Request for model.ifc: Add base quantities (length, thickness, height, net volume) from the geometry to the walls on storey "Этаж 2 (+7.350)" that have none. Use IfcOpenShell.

First a look at what the model holds.

```python
import ifcopenshell
import ifcopenshell.util.element
import ifcopenshell.util.unit

model = ifcopenshell.open("model.ifc")
print(model.schema)
for unit_type in ("LENGTHUNIT", "AREAUNIT", "VOLUMEUNIT"):
    print(unit_type, ifcopenshell.util.unit.calculate_unit_scale(model, unit_type))
storey = next(s for s in model.by_type("IfcBuildingStorey") if s.Name == "Этаж 2 (+7.350)")
walls = [e for e in ifcopenshell.util.element.get_decomposition(storey) if e.is_a("IfcWall")]
for e in sorted(walls, key=lambda e: e.id()):
    print(e.id(), e.is_a(), e.Name, list(ifcopenshell.util.element.get_psets(e, qtos_only=True)), sep=" | ")
```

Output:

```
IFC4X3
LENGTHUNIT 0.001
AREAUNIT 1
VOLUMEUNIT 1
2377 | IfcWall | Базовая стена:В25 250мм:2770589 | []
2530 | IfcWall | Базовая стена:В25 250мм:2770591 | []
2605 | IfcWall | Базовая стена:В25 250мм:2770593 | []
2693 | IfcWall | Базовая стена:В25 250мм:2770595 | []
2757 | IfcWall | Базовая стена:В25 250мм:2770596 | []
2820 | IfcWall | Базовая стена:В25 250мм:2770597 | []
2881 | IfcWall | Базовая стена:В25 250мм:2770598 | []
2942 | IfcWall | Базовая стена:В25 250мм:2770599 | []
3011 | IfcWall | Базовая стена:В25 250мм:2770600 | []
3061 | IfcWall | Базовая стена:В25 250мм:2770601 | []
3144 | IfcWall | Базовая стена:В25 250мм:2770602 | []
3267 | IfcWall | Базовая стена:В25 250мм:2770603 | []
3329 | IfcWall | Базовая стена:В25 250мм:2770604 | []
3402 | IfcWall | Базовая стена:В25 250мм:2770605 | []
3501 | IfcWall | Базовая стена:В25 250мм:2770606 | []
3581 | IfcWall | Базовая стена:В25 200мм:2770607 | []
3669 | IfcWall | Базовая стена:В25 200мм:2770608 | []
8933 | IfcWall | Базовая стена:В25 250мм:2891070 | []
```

```python
import ifcopenshell
import ifcopenshell.api.pset
import ifcopenshell.geom
import ifcopenshell.util.element
import ifcopenshell.util.shape
import ifcopenshell.util.unit

model = ifcopenshell.open("model.ifc")
unit_scale = ifcopenshell.util.unit.calculate_unit_scale(model)
volume_scale = ifcopenshell.util.unit.calculate_unit_scale(model, "VOLUMEUNIT")
settings = ifcopenshell.geom.settings()

storey = next(s for s in model.by_type("IfcBuildingStorey") if s.Name == "Этаж 2 (+7.350)")
walls = [e for e in ifcopenshell.util.element.get_decomposition(storey) if e.is_a("IfcWall")]

for e in sorted(walls, key=lambda e: e.id()):
    if ifcopenshell.util.element.get_psets(e, qtos_only=True, should_inherit=False):
        continue
    # Geometry comes back in metres, in the element's own axes.
    shape = ifcopenshell.geom.create_shape(settings, e)
    values = {
        "Length": ifcopenshell.util.shape.get_x(shape.geometry) / unit_scale,
        "Width": ifcopenshell.util.shape.get_y(shape.geometry) / unit_scale,
        "Height": ifcopenshell.util.shape.get_z(shape.geometry) / unit_scale,
        "NetVolume": ifcopenshell.util.shape.get_volume(shape.geometry) / volume_scale,
    }
    qto = ifcopenshell.api.pset.add_qto(model, product=e, name="Qto_WallBaseQuantities")
    ifcopenshell.api.pset.edit_qto(model, qto=qto, properties=values)
    print(e.id(), {k: round(v, 3) for k, v in values.items()})

model.write("model-out.ifc")
```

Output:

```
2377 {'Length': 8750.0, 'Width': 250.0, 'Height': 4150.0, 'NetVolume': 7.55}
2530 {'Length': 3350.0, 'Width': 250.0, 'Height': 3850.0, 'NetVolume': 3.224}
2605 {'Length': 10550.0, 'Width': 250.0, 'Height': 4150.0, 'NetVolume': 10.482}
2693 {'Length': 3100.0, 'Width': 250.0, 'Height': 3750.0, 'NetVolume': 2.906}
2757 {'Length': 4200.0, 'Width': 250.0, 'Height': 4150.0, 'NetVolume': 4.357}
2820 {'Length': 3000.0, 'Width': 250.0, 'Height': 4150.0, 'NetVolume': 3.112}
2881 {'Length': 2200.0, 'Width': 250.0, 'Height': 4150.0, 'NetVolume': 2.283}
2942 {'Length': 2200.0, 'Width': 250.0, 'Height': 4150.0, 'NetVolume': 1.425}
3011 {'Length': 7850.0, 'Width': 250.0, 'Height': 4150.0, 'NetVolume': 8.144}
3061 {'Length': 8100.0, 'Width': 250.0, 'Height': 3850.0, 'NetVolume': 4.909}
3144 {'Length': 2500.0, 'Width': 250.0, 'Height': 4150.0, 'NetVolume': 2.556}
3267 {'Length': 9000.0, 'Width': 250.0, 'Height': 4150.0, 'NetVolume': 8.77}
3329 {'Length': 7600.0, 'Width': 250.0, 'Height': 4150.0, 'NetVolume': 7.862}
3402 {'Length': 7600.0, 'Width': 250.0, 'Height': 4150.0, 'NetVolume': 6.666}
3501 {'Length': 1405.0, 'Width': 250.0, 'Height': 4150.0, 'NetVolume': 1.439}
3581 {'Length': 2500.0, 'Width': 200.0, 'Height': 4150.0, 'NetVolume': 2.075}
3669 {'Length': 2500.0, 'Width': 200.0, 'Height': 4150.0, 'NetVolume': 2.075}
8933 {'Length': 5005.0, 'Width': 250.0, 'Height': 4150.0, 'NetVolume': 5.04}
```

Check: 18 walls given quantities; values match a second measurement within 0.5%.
